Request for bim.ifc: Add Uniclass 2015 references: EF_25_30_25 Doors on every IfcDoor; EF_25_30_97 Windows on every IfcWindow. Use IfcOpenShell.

First a look at what the model holds.

```python
import ifcopenshell

model = ifcopenshell.open("bim.ifc")
print(model.schema)
print("classifications:", [c.Name for c in model.by_type("IfcClassification")])
for ifc_class in ("IfcDoor", "IfcRoof", "IfcStair", "IfcWall", "IfcWindow"):
    print(ifc_class, len(model.by_type(ifc_class)))
```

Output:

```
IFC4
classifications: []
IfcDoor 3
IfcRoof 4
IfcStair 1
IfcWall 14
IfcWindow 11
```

```python
import ifcopenshell
import ifcopenshell.api.classification

model = ifcopenshell.open("bim.ifc")

system = ifcopenshell.api.classification.add_classification(model, classification="Uniclass 2015")

codes = {
    "IfcDoor": ("EF_25_30_25", "Doors"),
    "IfcWindow": ("EF_25_30_97", "Windows"),
}
for ifc_class, (code, name) in codes.items():
    products = model.by_type(ifc_class)
    ifcopenshell.api.classification.add_reference(
        model, products=products, classification=system, identification=code, name=name
    )
    print(code, len(products))

model.write("bim-out.ifc")
```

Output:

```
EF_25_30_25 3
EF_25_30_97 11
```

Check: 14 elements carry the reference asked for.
